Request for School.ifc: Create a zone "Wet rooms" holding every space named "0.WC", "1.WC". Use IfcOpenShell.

First a look at what the model holds.

```python
import ifcopenshell

model = ifcopenshell.open("School.ifc")
print(model.schema)
seen = {}
for space in model.by_type("IfcSpace"):
    seen[space.LongName] = seen.get(space.LongName, 0) + 1
for name, count in sorted(seen.items(), key=str):
    print(count, "x", name)
print("zones:", [z.Name for z in model.by_type("IfcZone")][:20])
```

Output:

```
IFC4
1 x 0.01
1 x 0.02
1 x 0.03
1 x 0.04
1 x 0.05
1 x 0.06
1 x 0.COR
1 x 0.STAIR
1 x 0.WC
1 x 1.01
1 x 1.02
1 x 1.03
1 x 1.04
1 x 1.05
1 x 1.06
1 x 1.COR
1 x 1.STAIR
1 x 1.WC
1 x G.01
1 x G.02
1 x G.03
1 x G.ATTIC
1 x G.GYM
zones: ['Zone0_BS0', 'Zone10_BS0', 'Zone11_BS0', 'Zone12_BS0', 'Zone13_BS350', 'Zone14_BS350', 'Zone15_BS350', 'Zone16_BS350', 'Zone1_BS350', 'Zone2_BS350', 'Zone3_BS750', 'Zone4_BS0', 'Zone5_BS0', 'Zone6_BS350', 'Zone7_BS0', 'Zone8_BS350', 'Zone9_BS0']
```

```python
import ifcopenshell
import ifcopenshell.api.group
import ifcopenshell.api.root

model = ifcopenshell.open("School.ifc")

names = {"0.WC", "1.WC"}
spaces = [s for s in model.by_type("IfcSpace") if s.LongName in names]

zone = ifcopenshell.api.root.create_entity(model, ifc_class="IfcZone", name="Wet rooms")
ifcopenshell.api.group.assign_group(model, products=spaces, group=zone)
print(len(spaces), "spaces in", zone.Name)

model.write("School_v2.ifc")
```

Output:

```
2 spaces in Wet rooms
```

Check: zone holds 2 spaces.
